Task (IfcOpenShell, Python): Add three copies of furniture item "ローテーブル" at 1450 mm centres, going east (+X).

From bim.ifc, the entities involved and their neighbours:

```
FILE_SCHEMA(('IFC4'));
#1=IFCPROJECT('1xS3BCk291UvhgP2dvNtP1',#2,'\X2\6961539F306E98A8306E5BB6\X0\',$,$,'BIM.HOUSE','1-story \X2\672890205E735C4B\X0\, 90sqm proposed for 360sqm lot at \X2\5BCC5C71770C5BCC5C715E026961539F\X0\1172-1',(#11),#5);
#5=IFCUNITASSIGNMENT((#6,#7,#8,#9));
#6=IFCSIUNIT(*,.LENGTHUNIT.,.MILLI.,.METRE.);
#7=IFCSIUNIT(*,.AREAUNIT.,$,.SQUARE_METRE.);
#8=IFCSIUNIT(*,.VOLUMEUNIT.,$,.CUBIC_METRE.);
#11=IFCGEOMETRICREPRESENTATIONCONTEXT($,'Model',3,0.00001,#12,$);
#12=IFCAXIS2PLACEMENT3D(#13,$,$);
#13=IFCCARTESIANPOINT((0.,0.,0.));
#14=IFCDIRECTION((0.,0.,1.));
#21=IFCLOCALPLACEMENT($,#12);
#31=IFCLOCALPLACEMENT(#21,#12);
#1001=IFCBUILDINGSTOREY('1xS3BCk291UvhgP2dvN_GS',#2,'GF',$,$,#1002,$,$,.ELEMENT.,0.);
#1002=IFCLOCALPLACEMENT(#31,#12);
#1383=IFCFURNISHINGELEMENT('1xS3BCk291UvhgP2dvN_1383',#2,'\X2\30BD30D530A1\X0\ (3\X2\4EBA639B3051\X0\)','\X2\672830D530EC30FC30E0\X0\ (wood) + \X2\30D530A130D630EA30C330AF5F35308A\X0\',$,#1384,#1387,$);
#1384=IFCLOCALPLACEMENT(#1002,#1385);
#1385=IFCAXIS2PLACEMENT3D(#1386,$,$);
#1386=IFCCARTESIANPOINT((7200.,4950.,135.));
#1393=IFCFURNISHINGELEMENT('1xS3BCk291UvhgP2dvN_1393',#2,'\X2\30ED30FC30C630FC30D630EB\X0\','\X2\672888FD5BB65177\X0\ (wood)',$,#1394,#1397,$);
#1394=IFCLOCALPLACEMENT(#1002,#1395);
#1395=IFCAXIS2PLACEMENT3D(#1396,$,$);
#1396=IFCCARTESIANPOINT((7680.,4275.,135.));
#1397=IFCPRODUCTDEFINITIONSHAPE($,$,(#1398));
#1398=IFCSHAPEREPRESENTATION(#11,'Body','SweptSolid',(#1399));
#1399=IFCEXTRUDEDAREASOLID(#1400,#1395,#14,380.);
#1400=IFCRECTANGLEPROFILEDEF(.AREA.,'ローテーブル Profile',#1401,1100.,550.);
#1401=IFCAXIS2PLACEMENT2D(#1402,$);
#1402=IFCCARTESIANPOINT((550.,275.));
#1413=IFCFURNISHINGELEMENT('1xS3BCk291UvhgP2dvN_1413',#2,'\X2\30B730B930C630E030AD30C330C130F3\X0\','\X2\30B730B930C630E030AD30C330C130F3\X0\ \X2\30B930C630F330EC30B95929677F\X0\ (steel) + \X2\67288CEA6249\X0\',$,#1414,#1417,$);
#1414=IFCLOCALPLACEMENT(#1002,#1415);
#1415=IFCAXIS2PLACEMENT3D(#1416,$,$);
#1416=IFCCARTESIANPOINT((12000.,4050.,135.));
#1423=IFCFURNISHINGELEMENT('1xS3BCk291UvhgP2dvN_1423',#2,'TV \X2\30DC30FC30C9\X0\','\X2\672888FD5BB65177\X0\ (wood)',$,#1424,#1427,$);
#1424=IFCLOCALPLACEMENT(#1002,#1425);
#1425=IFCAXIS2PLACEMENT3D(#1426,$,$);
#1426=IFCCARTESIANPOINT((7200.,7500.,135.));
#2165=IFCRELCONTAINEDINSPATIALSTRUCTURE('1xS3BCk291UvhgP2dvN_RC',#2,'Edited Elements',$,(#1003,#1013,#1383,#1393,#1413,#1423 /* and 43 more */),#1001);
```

```python
import numpy as np
import ifcopenshell
import ifcopenshell.api.geometry
import ifcopenshell.api.root
import ifcopenshell.util.element
import ifcopenshell.util.placement

model = ifcopenshell.open("bim.ifc")


def reuse_history(source, copy):
    """copy_class also copies each property set's owner history, people and application; keep the originals."""
    for rel in copy.IsDefinedBy:
        if rel.is_a("IfcRelDefinesByProperties") and (history := rel.RelatingPropertyDefinition.OwnerHistory):
            rel.RelatingPropertyDefinition.OwnerHistory = source.OwnerHistory
            ifcopenshell.util.element.remove_deep2(model, history)


source = model.by_guid("1xS3BCk291UvhgP2dvN_1393")
base = ifcopenshell.util.placement.get_local_placement(source.ObjectPlacement)
step = np.array([1.0, 0.0, 0.0]) * 1450.0

for i in range(1, 4):
    copy = ifcopenshell.api.root.copy_class(model, product=source)
    copy.Representation = ifcopenshell.util.element.copy_deep(
        model, source.Representation, exclude=["IfcGeometricRepresentationContext", "IfcRepresentationMap"]
    )
    reuse_history(source, copy)
    matrix = base.copy()
    matrix[:3, 3] += i * step
    print("added at", matrix[:3, 3].round(3) + 0.0)
    ifcopenshell.api.geometry.edit_object_placement(model, product=copy, matrix=matrix, is_si=False)

model.write("bim_edited.ifc")
```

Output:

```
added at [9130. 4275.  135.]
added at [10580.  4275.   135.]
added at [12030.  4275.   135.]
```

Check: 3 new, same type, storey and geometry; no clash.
